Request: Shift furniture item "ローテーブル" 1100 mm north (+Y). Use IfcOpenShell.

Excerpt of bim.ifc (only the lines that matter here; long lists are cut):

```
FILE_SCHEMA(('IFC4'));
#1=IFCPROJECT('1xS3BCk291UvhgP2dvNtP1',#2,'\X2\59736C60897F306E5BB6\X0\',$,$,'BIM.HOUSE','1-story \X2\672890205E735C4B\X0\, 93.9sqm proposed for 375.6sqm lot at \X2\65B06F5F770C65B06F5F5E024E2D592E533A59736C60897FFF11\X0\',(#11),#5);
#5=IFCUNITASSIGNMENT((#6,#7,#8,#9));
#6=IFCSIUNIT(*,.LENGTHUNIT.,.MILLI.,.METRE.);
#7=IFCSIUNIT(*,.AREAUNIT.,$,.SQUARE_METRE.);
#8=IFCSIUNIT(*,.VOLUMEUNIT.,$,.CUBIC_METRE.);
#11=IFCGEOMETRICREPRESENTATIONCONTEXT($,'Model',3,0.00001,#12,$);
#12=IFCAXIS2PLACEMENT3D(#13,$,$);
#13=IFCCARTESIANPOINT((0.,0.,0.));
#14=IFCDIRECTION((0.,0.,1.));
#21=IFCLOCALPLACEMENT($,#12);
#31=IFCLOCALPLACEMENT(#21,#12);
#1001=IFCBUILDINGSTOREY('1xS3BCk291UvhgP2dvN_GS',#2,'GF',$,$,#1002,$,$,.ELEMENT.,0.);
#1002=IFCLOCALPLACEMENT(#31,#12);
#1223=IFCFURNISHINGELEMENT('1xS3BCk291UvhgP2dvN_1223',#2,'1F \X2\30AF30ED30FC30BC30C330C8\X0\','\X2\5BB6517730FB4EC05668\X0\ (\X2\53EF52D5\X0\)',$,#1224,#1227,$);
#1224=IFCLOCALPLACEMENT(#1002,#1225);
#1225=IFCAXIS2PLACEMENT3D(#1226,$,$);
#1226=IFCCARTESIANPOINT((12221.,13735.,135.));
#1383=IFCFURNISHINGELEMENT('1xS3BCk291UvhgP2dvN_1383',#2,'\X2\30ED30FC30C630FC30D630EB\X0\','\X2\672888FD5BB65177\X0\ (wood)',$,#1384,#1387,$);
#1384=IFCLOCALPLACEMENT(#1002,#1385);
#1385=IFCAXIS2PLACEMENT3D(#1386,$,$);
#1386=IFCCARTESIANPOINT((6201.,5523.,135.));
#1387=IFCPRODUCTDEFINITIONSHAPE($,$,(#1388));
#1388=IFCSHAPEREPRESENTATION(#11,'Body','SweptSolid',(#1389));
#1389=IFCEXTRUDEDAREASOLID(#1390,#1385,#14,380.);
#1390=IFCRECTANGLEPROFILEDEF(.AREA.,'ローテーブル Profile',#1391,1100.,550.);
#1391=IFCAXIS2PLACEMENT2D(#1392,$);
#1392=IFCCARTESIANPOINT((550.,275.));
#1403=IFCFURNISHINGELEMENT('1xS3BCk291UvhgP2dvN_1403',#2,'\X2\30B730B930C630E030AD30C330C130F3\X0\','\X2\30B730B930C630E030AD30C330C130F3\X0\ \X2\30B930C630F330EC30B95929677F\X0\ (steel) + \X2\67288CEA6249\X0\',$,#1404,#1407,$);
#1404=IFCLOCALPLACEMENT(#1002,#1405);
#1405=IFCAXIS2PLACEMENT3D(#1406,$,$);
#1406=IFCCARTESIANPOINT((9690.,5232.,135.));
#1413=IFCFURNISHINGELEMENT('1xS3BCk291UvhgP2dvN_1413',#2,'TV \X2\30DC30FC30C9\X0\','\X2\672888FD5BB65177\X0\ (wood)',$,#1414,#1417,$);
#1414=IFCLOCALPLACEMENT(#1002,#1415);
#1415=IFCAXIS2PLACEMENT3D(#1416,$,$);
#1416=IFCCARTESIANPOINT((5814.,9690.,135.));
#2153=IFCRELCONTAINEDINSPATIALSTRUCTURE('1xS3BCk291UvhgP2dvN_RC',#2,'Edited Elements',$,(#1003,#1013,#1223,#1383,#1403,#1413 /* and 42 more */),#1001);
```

```python
import ifcopenshell
import ifcopenshell.api.geometry
import ifcopenshell.util.placement

model = ifcopenshell.open("bim.ifc")

item = model.by_guid("1xS3BCk291UvhgP2dvN_1383")
matrix = ifcopenshell.util.placement.get_local_placement(item.ObjectPlacement)
matrix[1, 3] += 1100.0
ifcopenshell.api.geometry.edit_object_placement(model, product=item, matrix=matrix, is_si=False)

print(ifcopenshell.util.placement.get_local_placement(item.ObjectPlacement).round(3) + 0.0)

model.write("bim_rev.ifc")
```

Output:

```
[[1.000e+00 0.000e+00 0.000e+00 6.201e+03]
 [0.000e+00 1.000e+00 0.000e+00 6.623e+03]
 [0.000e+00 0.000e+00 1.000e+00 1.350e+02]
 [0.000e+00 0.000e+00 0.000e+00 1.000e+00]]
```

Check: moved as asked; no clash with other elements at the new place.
